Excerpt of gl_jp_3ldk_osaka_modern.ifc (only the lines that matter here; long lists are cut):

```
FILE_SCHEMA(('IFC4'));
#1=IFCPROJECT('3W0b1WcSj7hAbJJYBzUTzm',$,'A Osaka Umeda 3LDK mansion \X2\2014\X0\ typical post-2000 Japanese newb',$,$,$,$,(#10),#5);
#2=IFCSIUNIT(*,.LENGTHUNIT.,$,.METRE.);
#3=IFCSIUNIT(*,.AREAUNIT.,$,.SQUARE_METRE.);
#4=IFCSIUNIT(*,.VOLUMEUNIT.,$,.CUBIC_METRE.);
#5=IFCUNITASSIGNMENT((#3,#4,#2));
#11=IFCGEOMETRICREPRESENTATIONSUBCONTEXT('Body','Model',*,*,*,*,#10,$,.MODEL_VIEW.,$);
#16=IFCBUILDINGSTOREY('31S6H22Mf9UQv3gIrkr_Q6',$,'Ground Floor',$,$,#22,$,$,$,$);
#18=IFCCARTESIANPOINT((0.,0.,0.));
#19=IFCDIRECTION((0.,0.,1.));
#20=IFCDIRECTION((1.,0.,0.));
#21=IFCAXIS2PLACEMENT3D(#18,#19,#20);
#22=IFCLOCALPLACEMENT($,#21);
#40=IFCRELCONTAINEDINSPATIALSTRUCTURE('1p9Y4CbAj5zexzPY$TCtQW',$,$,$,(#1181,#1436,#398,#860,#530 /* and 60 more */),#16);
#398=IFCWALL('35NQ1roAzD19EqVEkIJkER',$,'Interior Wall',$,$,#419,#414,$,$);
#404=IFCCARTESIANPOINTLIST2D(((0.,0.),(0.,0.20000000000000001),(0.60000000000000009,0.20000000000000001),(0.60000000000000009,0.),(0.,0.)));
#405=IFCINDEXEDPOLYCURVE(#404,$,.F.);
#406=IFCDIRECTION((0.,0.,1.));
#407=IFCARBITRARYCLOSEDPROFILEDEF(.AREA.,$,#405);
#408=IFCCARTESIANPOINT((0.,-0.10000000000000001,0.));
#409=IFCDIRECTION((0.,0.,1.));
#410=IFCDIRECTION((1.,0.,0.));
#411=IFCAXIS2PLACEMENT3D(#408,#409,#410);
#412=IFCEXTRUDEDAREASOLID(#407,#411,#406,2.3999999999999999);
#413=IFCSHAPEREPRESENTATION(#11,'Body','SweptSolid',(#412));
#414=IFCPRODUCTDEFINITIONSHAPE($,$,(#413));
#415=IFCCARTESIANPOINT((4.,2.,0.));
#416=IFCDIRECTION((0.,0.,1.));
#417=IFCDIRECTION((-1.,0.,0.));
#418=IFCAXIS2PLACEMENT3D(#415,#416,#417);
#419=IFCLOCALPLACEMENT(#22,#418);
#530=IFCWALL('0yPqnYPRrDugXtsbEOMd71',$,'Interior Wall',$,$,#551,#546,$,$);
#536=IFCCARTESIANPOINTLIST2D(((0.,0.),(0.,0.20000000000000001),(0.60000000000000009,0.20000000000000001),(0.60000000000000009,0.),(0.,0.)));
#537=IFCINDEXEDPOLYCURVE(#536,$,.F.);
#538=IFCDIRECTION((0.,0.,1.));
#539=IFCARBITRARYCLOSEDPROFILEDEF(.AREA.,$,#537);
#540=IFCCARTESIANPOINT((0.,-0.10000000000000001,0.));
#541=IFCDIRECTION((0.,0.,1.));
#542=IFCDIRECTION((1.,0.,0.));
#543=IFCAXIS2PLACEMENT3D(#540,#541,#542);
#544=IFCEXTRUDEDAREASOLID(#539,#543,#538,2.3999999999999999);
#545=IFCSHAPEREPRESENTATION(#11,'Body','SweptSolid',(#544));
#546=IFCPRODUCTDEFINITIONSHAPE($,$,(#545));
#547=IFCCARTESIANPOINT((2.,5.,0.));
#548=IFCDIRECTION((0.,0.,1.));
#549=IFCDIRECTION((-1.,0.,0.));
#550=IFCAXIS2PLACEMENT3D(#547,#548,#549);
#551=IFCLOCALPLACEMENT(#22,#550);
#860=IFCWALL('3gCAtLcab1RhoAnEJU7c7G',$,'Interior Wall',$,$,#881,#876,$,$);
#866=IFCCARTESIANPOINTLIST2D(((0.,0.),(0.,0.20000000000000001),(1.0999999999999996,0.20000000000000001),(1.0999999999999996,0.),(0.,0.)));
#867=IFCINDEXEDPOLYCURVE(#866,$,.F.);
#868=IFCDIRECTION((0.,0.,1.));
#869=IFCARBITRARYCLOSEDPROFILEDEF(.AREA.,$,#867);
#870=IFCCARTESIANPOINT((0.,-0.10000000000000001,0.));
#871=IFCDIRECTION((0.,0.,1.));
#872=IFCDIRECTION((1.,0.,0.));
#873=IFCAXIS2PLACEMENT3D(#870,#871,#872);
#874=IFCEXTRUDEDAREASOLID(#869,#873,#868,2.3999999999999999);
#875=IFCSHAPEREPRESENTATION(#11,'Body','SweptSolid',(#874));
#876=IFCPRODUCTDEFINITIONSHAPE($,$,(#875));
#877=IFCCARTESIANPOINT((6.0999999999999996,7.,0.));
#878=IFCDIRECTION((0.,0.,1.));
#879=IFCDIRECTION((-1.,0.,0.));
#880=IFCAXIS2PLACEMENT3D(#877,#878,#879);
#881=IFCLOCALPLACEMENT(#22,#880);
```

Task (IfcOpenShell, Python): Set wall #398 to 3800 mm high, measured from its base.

```python
import ifcopenshell
import ifcopenshell.geom
import ifcopenshell.util.representation
import ifcopenshell.util.shape
import ifcopenshell.util.unit

model = ifcopenshell.open("gl_jp_3ldk_osaka_modern.ifc")
unit_scale = ifcopenshell.util.unit.calculate_unit_scale(model)
settings = ifcopenshell.geom.settings()


def volume(element):
    """Net volume in cubic metres, openings subtracted."""
    shape = ifcopenshell.geom.create_shape(settings, element)
    return ifcopenshell.util.shape.get_volume(shape.geometry)


wall = model.by_guid("35NQ1roAzD19EqVEkIJkER")
before = volume(wall)

body = ifcopenshell.util.representation.get_representation(wall, "Model", "Body")
solid = body.Items[0]
old_height = solid.Depth
solid.Depth = 3.8 / unit_scale
after = volume(wall)

print(f"height {old_height:g} -> {solid.Depth:g}, volume {before:.3f} -> {after:.3f} m3")

model.write("gl_jp_3ldk_osaka_modern-out.ifc")
```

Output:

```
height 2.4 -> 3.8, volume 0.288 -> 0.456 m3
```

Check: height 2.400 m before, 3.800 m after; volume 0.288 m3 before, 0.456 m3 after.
